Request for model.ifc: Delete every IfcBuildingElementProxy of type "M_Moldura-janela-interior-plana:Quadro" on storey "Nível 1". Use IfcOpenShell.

First a look at what the model holds.

```python
import ifcopenshell
import ifcopenshell.util.element

model = ifcopenshell.open("model.ifc")
print(model.schema)
storey = next(s for s in model.by_type("IfcBuildingStorey") if s.Name == "Nível 1")
proxies = [e for e in ifcopenshell.util.element.get_decomposition(storey) if e.is_a("IfcBuildingElementProxy")]
seen = {}
for e in proxies:
    element_type = ifcopenshell.util.element.get_type(e)
    name = element_type.Name if element_type not in (None, e) else None
    seen[name] = seen.get(name, 0) + 1
for name, count in sorted(seen.items(), key=str):
    print(count, "x", name)
```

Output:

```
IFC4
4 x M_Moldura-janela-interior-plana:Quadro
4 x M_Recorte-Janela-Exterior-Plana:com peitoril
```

```python
import ifcopenshell
import ifcopenshell.api.root
import ifcopenshell.util.element

model = ifcopenshell.open("model.ifc")

storey = next(s for s in model.by_type("IfcBuildingStorey") if s.Name == "Nível 1")
proxies = [e for e in ifcopenshell.util.element.get_decomposition(storey) if e.is_a("IfcBuildingElementProxy")]
targets = [e for e in proxies if (t := ifcopenshell.util.element.get_type(e)) not in (None, e) and t.Name == "M_Moldura-janela-interior-plana:Quadro"]

for e in targets:
    ifcopenshell.api.root.remove_product(model, product=e)
print(len(targets), "removed")

model.write("model-out.ifc")
```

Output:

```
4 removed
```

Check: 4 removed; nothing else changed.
